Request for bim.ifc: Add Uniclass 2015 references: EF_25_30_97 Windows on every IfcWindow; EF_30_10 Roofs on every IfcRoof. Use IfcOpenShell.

First a look at what the model holds.

```python
import ifcopenshell

model = ifcopenshell.open("bim.ifc")
print(model.schema)
print("classifications:", [c.Name for c in model.by_type("IfcClassification")])
for ifc_class in ("IfcDoor", "IfcRoof", "IfcStair", "IfcWall", "IfcWindow"):
    print(ifc_class, len(model.by_type(ifc_class)))
```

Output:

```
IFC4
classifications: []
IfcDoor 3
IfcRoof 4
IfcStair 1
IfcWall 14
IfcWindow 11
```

```python
import ifcopenshell
import ifcopenshell.api.classification

model = ifcopenshell.open("bim.ifc")

system = ifcopenshell.api.classification.add_classification(model, classification="Uniclass 2015")

codes = {
    "IfcWindow": ("EF_25_30_97", "Windows"),
    "IfcRoof": ("EF_30_10", "Roofs"),
}
for ifc_class, (code, name) in codes.items():
    products = model.by_type(ifc_class)
    ifcopenshell.api.classification.add_reference(
        model, products=products, classification=system, identification=code, name=name
    )
    print(code, len(products))

model.write("bim_edited.ifc")
```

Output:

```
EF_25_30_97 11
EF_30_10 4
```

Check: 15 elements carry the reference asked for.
